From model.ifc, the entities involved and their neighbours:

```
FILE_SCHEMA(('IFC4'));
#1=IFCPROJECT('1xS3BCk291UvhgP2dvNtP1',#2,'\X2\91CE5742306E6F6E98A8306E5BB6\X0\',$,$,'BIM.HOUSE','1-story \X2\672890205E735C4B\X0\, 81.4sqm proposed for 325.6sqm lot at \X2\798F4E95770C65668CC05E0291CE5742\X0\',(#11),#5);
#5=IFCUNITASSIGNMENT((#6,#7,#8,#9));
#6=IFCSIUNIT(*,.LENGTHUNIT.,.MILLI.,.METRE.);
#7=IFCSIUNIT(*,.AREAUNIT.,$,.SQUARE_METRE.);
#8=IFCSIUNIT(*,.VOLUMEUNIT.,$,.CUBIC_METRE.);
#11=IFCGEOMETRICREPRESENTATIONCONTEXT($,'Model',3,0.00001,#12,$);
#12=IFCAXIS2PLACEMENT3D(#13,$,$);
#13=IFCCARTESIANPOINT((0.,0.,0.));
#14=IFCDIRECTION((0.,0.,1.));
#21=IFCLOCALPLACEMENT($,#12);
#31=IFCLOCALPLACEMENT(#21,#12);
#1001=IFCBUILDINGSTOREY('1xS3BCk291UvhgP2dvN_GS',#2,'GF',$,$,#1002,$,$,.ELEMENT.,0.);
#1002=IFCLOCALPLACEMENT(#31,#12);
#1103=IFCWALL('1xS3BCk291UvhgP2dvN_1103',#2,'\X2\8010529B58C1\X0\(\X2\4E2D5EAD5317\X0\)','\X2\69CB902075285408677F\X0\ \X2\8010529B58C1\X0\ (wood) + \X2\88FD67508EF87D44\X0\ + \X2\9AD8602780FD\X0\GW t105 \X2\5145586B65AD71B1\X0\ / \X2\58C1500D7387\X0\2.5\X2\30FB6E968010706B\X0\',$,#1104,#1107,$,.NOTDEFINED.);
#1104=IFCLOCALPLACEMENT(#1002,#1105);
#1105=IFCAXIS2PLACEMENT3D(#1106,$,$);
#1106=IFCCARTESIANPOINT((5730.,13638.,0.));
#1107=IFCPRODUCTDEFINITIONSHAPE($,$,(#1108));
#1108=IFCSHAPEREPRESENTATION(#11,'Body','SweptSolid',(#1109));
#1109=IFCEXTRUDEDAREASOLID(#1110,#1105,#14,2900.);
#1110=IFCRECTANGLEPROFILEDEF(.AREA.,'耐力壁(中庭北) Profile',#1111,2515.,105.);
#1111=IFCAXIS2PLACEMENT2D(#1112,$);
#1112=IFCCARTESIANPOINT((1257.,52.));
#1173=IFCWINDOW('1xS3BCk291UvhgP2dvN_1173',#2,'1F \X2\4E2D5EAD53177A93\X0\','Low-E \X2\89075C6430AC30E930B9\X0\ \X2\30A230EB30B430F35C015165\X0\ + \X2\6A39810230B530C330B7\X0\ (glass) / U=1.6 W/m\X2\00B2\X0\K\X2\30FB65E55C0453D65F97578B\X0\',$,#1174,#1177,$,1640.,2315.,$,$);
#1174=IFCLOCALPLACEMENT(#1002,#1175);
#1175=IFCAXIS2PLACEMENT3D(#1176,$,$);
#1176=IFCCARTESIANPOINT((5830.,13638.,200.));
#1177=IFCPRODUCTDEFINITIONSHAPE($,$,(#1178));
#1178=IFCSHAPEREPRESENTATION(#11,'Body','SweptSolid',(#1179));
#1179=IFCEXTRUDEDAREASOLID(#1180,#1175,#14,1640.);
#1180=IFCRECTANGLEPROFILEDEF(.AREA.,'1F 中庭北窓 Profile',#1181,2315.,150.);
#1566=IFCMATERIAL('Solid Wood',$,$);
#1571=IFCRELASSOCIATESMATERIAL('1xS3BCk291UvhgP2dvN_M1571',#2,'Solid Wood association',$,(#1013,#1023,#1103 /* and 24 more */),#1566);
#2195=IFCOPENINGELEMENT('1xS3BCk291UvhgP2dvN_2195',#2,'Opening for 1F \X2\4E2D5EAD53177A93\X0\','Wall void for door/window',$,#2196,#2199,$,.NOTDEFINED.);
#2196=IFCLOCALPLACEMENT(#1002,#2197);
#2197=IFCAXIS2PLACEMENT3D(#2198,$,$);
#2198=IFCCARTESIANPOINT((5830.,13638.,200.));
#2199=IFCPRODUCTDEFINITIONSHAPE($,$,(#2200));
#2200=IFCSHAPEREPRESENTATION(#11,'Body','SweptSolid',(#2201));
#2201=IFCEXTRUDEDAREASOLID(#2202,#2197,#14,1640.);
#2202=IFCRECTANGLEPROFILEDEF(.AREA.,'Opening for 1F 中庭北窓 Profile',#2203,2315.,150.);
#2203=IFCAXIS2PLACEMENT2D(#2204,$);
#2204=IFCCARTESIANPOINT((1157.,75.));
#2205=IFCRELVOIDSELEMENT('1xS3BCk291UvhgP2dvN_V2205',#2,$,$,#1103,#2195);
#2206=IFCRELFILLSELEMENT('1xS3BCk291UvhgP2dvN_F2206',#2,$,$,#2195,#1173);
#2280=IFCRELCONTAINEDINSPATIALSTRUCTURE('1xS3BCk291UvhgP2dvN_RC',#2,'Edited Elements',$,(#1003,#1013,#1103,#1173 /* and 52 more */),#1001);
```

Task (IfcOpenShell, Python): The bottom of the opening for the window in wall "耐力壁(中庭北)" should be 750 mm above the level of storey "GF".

```python
import numpy as np
import ifcopenshell
import ifcopenshell.api.geometry
import ifcopenshell.geom
import ifcopenshell.util.element
import ifcopenshell.util.placement
import ifcopenshell.util.shape
import ifcopenshell.util.unit

model = ifcopenshell.open("model.ifc")
unit_scale = ifcopenshell.util.unit.calculate_unit_scale(model)

window = model.by_id(1173)
opening = window.FillsVoids[0].RelatingOpeningElement
storey = ifcopenshell.util.element.get_container(window, ifc_class="IfcBuildingStorey")
level = ifcopenshell.util.placement.get_local_placement(storey.ObjectPlacement)[2, 3]

# The opening's origin need not be at the sill, so measure its lowest point.
shape = ifcopenshell.geom.create_shape(ifcopenshell.geom.settings(), opening)
bottom = ifcopenshell.util.shape.get_shape_bottom_elevation(shape, shape.geometry) / unit_scale
dz = level + 750.0 - bottom

shift = np.array([0.0, 0.0, dz])
# The window is not placed relative to its opening, so move both.
for product in (opening, window):
    matrix = ifcopenshell.util.placement.get_local_placement(product.ObjectPlacement)
    matrix[:3, 3] += shift
    ifcopenshell.api.geometry.edit_object_placement(model, product=product, matrix=matrix, is_si=False)

print(f"moved by {dz * unit_scale:+.3f} m")

model.write("model_edited.ifc")
```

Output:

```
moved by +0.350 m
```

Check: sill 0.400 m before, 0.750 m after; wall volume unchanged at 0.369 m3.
